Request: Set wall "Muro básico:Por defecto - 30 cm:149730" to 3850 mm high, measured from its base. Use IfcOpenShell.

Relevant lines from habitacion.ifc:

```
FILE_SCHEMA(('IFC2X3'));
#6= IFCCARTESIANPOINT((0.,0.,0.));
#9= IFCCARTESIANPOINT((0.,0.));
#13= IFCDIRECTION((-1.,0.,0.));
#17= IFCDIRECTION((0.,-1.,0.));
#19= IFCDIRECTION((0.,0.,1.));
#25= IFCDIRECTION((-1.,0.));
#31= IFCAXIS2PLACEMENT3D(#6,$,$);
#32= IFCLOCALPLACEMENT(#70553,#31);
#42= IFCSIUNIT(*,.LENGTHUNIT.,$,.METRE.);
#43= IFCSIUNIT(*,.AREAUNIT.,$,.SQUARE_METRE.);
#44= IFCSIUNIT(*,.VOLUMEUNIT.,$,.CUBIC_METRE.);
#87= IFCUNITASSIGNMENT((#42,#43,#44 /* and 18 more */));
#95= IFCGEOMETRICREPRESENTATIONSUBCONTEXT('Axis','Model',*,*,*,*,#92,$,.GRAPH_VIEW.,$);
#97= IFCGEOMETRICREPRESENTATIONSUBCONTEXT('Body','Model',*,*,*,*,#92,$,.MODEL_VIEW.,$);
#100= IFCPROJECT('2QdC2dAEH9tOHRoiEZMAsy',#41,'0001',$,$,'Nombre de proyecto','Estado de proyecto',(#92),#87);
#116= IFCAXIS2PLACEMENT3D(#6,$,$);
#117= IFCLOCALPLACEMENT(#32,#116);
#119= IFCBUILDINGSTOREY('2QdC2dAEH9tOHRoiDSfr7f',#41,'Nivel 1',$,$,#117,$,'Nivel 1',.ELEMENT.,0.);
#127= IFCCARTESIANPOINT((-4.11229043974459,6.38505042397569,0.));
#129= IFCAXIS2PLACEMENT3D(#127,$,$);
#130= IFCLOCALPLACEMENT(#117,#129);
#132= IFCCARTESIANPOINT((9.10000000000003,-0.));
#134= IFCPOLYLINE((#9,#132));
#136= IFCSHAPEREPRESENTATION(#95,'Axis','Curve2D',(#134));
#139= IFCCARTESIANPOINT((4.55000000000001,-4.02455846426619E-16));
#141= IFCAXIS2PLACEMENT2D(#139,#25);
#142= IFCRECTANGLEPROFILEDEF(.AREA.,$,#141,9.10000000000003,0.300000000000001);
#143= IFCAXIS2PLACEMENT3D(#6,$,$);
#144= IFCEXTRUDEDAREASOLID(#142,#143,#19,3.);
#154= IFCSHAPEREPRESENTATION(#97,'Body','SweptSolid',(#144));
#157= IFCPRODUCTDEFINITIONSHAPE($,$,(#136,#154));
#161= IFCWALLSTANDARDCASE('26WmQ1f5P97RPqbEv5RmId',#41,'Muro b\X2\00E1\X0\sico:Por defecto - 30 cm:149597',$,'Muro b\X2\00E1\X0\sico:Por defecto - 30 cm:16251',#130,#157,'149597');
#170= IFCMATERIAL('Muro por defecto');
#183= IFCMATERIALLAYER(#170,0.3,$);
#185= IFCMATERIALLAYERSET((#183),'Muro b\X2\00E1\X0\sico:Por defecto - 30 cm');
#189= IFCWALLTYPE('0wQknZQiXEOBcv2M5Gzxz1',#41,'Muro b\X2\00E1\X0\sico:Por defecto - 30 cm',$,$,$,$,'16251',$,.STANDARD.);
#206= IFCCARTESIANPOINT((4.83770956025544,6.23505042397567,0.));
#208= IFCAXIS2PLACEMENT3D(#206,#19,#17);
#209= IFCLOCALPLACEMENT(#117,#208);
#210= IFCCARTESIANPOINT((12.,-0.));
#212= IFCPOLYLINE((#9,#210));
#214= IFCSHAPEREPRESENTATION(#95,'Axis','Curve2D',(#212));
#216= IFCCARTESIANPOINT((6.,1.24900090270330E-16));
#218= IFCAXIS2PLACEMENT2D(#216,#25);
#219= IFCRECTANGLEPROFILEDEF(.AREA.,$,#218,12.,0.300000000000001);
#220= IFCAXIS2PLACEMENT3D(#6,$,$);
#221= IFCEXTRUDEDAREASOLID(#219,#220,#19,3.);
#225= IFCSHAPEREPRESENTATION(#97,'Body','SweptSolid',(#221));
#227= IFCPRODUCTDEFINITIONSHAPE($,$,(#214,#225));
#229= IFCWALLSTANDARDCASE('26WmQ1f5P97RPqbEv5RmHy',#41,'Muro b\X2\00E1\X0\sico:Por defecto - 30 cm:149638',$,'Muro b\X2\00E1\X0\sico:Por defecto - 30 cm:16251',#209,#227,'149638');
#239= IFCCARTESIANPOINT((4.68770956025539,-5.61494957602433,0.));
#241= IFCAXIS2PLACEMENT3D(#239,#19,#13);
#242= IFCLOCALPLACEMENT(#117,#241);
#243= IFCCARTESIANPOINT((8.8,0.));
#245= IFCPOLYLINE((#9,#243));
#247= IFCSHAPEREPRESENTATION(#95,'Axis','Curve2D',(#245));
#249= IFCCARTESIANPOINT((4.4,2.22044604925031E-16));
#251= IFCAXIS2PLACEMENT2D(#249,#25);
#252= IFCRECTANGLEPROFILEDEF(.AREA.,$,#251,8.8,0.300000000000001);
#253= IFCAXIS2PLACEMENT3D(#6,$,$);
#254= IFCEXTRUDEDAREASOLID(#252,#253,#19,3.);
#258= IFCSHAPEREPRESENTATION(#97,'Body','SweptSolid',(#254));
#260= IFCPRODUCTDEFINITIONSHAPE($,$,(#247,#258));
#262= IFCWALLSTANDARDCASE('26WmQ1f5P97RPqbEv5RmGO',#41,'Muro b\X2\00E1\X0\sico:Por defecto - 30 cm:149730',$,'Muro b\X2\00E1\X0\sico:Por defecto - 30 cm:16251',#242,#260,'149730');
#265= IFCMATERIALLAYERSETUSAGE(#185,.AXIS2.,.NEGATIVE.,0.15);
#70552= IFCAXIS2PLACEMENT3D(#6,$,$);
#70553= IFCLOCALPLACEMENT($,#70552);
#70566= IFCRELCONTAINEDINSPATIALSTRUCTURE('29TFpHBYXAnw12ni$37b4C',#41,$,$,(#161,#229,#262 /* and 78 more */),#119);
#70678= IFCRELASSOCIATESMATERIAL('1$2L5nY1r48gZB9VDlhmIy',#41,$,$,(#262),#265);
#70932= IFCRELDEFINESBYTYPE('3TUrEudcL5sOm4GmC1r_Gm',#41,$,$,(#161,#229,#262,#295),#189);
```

```python
import ifcopenshell
import ifcopenshell.geom
import ifcopenshell.util.representation
import ifcopenshell.util.shape
import ifcopenshell.util.unit

model = ifcopenshell.open("habitacion.ifc")
unit_scale = ifcopenshell.util.unit.calculate_unit_scale(model)
settings = ifcopenshell.geom.settings()


def volume(element):
    """Net volume in cubic metres, openings subtracted."""
    shape = ifcopenshell.geom.create_shape(settings, element)
    return ifcopenshell.util.shape.get_volume(shape.geometry)


wall = model.by_id(262)
before = volume(wall)

body = ifcopenshell.util.representation.get_representation(wall, "Model", "Body")
solid = body.Items[0]
old_height = solid.Depth
solid.Depth = 3.85 / unit_scale
after = volume(wall)

print(f"height {old_height:g} -> {solid.Depth:g}, volume {before:.3f} -> {after:.3f} m3")

model.write("habitacion-out.ifc")
```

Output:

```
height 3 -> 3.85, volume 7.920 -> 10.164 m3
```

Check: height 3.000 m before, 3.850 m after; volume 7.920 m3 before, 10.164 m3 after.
